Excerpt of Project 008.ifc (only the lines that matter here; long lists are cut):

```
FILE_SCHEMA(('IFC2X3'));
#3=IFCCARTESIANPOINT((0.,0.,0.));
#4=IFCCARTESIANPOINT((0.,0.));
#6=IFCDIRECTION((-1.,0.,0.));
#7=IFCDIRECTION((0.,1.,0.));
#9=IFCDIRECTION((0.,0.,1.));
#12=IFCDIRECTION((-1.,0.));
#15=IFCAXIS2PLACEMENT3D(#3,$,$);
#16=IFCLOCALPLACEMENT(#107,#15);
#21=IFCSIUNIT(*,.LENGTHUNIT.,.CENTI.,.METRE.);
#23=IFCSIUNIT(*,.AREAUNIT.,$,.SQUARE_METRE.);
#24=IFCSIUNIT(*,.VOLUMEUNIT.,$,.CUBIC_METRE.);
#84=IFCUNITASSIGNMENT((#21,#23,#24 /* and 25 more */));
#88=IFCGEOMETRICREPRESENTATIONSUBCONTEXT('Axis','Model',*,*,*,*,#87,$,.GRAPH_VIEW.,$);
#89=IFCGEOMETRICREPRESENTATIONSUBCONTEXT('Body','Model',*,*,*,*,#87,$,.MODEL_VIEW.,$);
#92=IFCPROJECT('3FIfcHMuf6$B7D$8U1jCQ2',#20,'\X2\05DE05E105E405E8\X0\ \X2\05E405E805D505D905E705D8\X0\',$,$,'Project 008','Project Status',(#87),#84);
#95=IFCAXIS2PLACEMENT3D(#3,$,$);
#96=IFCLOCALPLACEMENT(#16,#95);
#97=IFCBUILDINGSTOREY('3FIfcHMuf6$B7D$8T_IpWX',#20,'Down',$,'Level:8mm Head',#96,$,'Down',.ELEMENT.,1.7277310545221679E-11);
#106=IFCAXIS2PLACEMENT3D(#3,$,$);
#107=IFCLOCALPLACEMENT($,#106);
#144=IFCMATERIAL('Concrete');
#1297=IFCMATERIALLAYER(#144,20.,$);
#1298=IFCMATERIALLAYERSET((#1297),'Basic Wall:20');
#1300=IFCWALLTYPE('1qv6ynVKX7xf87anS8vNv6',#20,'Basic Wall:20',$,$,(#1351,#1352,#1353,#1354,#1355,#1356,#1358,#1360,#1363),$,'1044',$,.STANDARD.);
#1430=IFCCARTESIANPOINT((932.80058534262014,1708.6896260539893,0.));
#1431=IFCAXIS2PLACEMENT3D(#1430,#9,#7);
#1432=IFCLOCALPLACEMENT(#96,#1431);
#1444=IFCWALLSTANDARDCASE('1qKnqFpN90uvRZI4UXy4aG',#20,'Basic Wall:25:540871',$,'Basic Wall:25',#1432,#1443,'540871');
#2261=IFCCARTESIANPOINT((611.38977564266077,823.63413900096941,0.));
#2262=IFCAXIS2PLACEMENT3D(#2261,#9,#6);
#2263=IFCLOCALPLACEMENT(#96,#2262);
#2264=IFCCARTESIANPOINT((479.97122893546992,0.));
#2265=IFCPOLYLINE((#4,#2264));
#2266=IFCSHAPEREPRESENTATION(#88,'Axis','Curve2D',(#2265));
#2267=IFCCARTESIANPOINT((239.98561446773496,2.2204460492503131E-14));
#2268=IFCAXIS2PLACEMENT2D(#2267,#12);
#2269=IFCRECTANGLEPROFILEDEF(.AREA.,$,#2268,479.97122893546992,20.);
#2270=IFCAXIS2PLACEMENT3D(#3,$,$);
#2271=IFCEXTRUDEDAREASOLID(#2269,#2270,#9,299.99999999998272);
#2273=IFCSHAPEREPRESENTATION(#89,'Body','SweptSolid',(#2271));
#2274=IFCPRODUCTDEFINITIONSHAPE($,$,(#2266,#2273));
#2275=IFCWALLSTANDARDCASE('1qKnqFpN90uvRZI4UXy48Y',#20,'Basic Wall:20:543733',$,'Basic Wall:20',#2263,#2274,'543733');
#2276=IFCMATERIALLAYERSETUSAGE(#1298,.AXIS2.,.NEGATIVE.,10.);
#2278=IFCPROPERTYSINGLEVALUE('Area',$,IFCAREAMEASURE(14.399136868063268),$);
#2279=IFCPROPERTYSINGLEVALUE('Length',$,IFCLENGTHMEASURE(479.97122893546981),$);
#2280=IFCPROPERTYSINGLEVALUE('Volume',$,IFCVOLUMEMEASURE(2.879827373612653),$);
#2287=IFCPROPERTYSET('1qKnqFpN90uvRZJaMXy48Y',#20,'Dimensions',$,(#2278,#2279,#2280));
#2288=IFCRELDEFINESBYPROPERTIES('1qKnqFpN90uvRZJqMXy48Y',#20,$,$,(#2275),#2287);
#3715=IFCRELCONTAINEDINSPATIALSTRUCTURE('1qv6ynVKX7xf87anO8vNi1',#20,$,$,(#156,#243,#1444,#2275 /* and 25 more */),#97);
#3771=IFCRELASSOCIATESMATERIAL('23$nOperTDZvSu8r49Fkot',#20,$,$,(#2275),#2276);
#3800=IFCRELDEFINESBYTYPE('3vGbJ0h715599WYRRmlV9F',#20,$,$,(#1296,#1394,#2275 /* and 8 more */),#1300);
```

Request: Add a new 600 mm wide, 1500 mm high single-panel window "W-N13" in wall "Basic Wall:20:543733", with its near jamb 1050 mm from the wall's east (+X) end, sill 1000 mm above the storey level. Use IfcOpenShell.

```python
import numpy as np
import ifcopenshell
import ifcopenshell.api.feature
import ifcopenshell.api.geometry
import ifcopenshell.api.pset
import ifcopenshell.api.root
import ifcopenshell.api.spatial
import ifcopenshell.api.type
import ifcopenshell.geom
import ifcopenshell.util.element
import ifcopenshell.util.placement
import ifcopenshell.util.representation
import ifcopenshell.util.shape
import ifcopenshell.util.unit

model = ifcopenshell.open("Project 008.ifc")
unit_scale = ifcopenshell.util.unit.calculate_unit_scale(model)
area_scale = ifcopenshell.util.unit.calculate_unit_scale(model, "AREAUNIT")
volume_scale = ifcopenshell.util.unit.calculate_unit_scale(model, "VOLUMEUNIT")
settings = ifcopenshell.geom.settings()


def volume(element):
    """Net volume in cubic metres, openings subtracted."""
    shape = ifcopenshell.geom.create_shape(settings, element)
    return ifcopenshell.util.shape.get_volume(shape.geometry)


wall = model.by_guid("1qKnqFpN90uvRZI4UXy48Y")
storey = ifcopenshell.util.element.get_container(wall, ifc_class="IfcBuildingStorey")
context = ifcopenshell.util.representation.get_context(model, "Model", "Body", "MODEL_VIEW")
before = volume(wall)

width, height, from_end, sill = 0.6, 1.5, 1.05, 1  # metres

# The wall runs along its own X axis, and the end named is its -X end.
wall_shape = ifcopenshell.geom.create_shape(settings, wall)
x, y, z = ifcopenshell.util.shape.get_vertices(wall_shape.geometry).T
start = x.min() + from_end
face, thickness = float(y.min()), float(y.max() - y.min())
wall_matrix = ifcopenshell.util.placement.get_local_placement(wall.ObjectPlacement)
level = ifcopenshell.util.placement.get_local_placement(storey.ObjectPlacement)[2, 3]


def in_wall(x, y):
    """Placement at x, y metres in the wall's axes, at sill height."""
    matrix = wall_matrix.copy()
    matrix[:, 3] = wall_matrix @ np.array([x / unit_scale, y / unit_scale, 0.0, 1.0])
    matrix[2, 3] = level + sill / unit_scale
    return matrix


# Opening: a box that overshoots both wall faces by 50 mm.
opening = ifcopenshell.api.root.create_entity(model, ifc_class="IfcOpeningElement")
box = ifcopenshell.api.geometry.add_wall_representation(
    model, context=context, length=width, height=height, thickness=thickness + 0.1
)
ifcopenshell.api.geometry.assign_representation(model, product=opening, representation=box)
ifcopenshell.api.geometry.edit_object_placement(model, product=opening, matrix=in_wall(start, face - 0.05), is_si=False)
ifcopenshell.api.feature.add_feature(model, feature=opening, element=wall)

window = ifcopenshell.api.root.create_entity(model, ifc_class="IfcWindow", name="W-N13")
window.OverallWidth, window.OverallHeight = width / unit_scale, height / unit_scale
body = ifcopenshell.api.geometry.add_window_representation(
    model,
    context=context,
    overall_width=window.OverallWidth,
    overall_height=window.OverallHeight,
    partition_type="SINGLE_PANEL",
)
ifcopenshell.api.geometry.assign_representation(model, product=window, representation=body)
ifcopenshell.api.spatial.assign_container(model, products=[window], relating_structure=storey)
fills = ifcopenshell.api.feature.add_filling(model, opening=opening, element=window)
fills.OwnerHistory = window.OwnerHistory  # required in IFC2X3

# IFC2X3 keeps the operation on the window style.
style = ifcopenshell.api.root.create_entity(model, ifc_class="IfcWindowStyle", name="W-N13")
style.OperationType, style.ConstructionType = "SINGLE_PANEL", "NOTDEFINED"
style.ParameterTakesPrecedence = style.Sizeable = False
ifcopenshell.api.type.assign_type(model, related_objects=[window], relating_type=style)

# Centre the window in the wall's thickness.
ifcopenshell.api.geometry.edit_object_placement(model, product=window, matrix=in_wall(start, face), is_si=False)
window_shape = ifcopenshell.geom.create_shape(settings, window)
depth = ifcopenshell.util.shape.get_vertices(window_shape.geometry)[:, 1]
offset = face + thickness / 2 - (depth.min() + depth.max()) / 2
ifcopenshell.api.geometry.edit_object_placement(model, product=window, matrix=in_wall(start, offset), is_si=False)

after = volume(wall)

# Update the wall's stored quantities.
pset = model.by_id(ifcopenshell.util.element.get_pset(wall, "Dimensions", should_inherit=False)["id"])
ifcopenshell.api.pset.edit_pset(model, pset=pset, properties={
    "Area": model.create_entity("IfcAreaMeasure", after / thickness / area_scale),
    "Volume": model.create_entity("IfcVolumeMeasure", after / volume_scale),
})

print(f"wall volume {before:.3f} -> {after:.3f} m3")

model.write("Project 008_edited.ifc")
```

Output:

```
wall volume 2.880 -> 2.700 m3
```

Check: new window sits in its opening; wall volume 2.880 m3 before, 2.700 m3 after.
